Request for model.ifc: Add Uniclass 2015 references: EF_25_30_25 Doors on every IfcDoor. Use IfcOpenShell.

First a look at what the model holds.

```python
import ifcopenshell

model = ifcopenshell.open("model.ifc")
print(model.schema)
print("classifications:", [c.Name for c in model.by_type("IfcClassification")])
for ifc_class in ("IfcDoor", "IfcRoof", "IfcStair", "IfcWall", "IfcWindow"):
    print(ifc_class, len(model.by_type(ifc_class)))
```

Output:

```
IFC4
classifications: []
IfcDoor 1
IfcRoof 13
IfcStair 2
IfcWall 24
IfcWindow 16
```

```python
import ifcopenshell
import ifcopenshell.api.classification

model = ifcopenshell.open("model.ifc")

system = ifcopenshell.api.classification.add_classification(model, classification="Uniclass 2015")

codes = {
    "IfcDoor": ("EF_25_30_25", "Doors"),
}
for ifc_class, (code, name) in codes.items():
    products = model.by_type(ifc_class)
    ifcopenshell.api.classification.add_reference(
        model, products=products, classification=system, identification=code, name=name
    )
    print(code, len(products))

model.write("model_v2.ifc")
```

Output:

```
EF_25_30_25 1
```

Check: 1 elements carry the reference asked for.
